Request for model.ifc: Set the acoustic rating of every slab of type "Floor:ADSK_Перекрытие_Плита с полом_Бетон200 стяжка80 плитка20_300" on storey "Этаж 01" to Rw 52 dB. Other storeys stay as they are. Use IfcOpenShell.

First a look at what the model holds.

```python
import ifcopenshell
import ifcopenshell.util.element

model = ifcopenshell.open("model.ifc")
print(model.schema)
storey = next(s for s in model.by_type("IfcBuildingStorey") if s.Name == "Этаж 01")
slabs = [e for e in ifcopenshell.util.element.get_decomposition(storey) if e.is_a("IfcSlab")]
seen = {}
for e in slabs:
    element_type = ifcopenshell.util.element.get_type(e)
    key = (element_type.Name if element_type != e and element_type else None, ifcopenshell.util.element.get_pset(e, "Pset_SlabCommon", "AcousticRating"))
    seen[key] = seen.get(key, 0) + 1
for (name, value), count in sorted(seen.items(), key=str):
    print(count, "x", name, "|", value)
```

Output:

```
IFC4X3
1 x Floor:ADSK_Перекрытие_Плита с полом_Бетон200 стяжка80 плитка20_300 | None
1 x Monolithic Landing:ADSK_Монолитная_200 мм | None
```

```python
import ifcopenshell
import ifcopenshell.api.pset
import ifcopenshell.util.element

model = ifcopenshell.open("model.ifc")

storey = next(s for s in model.by_type("IfcBuildingStorey") if s.Name == "Этаж 01")
slabs = [e for e in ifcopenshell.util.element.get_decomposition(storey) if e.is_a("IfcSlab")]

count = 0
for e in slabs:
    element_type = ifcopenshell.util.element.get_type(e)
    if element_type in (None, e) or element_type.Name != "Floor:ADSK_Перекрытие_Плита с полом_Бетон200 стяжка80 плитка20_300":
        continue
    # add_pset returns the element's existing set when there is one.
    pset = ifcopenshell.api.pset.add_pset(model, product=e, name="Pset_SlabCommon")
    ifcopenshell.api.pset.edit_pset(model, pset=pset, properties={"AcousticRating": "Rw 52 dB"})
    count += 1

print(count, "slabs updated")

model.write("model_edited.ifc")
```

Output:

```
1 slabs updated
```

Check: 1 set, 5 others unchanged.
